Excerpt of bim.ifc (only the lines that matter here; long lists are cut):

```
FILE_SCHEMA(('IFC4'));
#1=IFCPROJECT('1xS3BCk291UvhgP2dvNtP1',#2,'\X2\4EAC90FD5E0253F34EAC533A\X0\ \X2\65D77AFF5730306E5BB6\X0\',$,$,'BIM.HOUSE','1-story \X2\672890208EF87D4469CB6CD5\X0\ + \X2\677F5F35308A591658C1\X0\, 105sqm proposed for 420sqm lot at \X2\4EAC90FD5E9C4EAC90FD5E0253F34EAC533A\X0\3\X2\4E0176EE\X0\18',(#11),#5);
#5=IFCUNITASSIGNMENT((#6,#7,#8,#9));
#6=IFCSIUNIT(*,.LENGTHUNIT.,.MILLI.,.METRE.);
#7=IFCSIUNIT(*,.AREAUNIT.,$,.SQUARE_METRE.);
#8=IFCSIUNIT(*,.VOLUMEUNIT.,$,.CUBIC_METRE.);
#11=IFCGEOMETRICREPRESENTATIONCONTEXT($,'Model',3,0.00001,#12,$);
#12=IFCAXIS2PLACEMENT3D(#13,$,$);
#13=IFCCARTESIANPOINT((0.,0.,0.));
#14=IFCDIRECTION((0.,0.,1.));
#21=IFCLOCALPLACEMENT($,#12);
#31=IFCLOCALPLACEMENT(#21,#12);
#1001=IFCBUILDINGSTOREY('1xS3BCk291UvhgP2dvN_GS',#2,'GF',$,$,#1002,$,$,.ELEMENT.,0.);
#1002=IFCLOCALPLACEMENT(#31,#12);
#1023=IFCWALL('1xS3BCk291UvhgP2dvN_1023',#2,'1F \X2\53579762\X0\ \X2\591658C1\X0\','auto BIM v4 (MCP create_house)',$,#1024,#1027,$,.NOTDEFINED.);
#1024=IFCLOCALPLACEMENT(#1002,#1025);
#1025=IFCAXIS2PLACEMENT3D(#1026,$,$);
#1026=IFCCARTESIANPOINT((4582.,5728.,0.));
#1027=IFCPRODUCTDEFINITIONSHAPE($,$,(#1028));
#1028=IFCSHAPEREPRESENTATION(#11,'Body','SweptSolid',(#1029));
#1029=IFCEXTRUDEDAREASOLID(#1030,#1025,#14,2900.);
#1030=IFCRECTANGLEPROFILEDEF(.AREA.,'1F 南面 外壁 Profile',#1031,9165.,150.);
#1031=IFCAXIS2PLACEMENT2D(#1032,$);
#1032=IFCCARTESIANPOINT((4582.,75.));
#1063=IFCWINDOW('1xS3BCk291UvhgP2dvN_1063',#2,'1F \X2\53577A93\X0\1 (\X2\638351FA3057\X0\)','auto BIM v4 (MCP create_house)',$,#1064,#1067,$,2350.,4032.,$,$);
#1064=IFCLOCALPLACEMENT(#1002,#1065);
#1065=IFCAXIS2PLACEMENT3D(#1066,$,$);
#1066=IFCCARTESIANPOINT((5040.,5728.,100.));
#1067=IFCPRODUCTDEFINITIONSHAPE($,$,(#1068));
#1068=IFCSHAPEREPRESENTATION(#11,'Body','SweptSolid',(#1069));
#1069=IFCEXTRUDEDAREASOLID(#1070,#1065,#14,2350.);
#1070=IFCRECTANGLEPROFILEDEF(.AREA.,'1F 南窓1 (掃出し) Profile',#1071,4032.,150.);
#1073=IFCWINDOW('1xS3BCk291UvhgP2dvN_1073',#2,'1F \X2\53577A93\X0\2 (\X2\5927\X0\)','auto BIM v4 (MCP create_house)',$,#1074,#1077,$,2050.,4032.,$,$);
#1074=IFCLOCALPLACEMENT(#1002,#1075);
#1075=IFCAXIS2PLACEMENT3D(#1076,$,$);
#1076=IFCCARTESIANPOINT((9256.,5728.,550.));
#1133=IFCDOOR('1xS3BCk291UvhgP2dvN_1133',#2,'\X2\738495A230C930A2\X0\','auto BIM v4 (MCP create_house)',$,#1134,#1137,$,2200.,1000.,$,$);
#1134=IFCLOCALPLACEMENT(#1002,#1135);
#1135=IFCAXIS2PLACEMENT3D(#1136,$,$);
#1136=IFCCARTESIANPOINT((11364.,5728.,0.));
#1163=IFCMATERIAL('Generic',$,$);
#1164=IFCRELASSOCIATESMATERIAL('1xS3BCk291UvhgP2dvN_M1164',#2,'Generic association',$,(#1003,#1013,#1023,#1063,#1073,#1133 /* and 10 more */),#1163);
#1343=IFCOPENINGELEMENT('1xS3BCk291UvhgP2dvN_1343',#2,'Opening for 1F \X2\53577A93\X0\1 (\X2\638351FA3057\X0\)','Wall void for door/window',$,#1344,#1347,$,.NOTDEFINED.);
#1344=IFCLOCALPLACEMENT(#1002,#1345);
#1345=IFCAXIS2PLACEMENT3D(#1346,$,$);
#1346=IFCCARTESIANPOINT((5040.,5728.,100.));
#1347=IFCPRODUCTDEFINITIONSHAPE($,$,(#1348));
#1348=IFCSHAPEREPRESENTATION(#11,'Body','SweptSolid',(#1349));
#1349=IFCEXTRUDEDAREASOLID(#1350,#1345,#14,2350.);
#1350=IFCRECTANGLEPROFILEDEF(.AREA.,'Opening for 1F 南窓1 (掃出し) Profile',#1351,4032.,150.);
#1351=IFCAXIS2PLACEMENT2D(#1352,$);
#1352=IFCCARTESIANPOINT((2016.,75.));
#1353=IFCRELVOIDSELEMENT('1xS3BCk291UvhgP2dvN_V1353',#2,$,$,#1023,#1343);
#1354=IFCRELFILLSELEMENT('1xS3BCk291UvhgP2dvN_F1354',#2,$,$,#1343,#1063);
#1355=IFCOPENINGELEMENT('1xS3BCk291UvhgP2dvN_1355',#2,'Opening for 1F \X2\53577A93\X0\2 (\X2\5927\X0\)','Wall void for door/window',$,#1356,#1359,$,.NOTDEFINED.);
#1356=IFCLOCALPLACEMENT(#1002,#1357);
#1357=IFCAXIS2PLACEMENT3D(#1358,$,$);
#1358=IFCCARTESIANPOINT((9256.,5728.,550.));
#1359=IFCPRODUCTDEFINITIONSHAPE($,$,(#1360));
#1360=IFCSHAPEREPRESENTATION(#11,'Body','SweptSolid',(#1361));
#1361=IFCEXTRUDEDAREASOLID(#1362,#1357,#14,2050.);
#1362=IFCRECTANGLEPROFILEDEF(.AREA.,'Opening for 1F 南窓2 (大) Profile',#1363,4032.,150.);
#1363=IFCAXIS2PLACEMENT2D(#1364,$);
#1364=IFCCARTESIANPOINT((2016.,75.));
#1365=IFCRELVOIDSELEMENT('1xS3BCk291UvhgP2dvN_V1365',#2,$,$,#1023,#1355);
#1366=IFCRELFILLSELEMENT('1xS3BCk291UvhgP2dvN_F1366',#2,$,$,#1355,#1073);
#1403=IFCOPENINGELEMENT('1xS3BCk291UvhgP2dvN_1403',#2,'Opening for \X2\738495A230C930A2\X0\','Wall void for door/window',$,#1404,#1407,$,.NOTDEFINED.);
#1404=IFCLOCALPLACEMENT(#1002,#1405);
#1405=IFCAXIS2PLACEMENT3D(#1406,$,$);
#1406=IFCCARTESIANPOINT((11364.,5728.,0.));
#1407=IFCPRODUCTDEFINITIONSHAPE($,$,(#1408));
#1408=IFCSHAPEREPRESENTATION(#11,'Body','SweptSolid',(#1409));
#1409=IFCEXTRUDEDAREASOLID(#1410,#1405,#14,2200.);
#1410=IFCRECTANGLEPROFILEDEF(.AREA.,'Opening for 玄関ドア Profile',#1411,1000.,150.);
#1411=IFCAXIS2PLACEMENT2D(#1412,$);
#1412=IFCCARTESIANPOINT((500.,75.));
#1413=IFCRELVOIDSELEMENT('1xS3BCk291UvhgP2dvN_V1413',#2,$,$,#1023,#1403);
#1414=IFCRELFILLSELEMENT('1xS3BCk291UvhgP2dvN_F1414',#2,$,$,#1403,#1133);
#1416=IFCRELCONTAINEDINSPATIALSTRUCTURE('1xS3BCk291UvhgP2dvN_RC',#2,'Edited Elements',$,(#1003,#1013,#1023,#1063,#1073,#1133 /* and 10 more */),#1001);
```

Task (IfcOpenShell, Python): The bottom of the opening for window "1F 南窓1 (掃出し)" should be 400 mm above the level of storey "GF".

```python
import numpy as np
import ifcopenshell
import ifcopenshell.api.geometry
import ifcopenshell.geom
import ifcopenshell.util.element
import ifcopenshell.util.placement
import ifcopenshell.util.shape
import ifcopenshell.util.unit

model = ifcopenshell.open("bim.ifc")
unit_scale = ifcopenshell.util.unit.calculate_unit_scale(model)

window = model.by_id(1063)
opening = window.FillsVoids[0].RelatingOpeningElement
storey = ifcopenshell.util.element.get_container(window, ifc_class="IfcBuildingStorey")
level = ifcopenshell.util.placement.get_local_placement(storey.ObjectPlacement)[2, 3]

# The opening's origin need not be at the sill, so measure its lowest point.
shape = ifcopenshell.geom.create_shape(ifcopenshell.geom.settings(), opening)
bottom = ifcopenshell.util.shape.get_shape_bottom_elevation(shape, shape.geometry) / unit_scale
dz = level + 400.0 - bottom

shift = np.array([0.0, 0.0, dz])
# The window is not placed relative to its opening, so move both.
for product in (opening, window):
    matrix = ifcopenshell.util.placement.get_local_placement(product.ObjectPlacement)
    matrix[:3, 3] += shift
    ifcopenshell.api.geometry.edit_object_placement(model, product=product, matrix=matrix, is_si=False)

print(f"moved by {dz * unit_scale:+.3f} m")

model.write("bim_v2.ifc")
```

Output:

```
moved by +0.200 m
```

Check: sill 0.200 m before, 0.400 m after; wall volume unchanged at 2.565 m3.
